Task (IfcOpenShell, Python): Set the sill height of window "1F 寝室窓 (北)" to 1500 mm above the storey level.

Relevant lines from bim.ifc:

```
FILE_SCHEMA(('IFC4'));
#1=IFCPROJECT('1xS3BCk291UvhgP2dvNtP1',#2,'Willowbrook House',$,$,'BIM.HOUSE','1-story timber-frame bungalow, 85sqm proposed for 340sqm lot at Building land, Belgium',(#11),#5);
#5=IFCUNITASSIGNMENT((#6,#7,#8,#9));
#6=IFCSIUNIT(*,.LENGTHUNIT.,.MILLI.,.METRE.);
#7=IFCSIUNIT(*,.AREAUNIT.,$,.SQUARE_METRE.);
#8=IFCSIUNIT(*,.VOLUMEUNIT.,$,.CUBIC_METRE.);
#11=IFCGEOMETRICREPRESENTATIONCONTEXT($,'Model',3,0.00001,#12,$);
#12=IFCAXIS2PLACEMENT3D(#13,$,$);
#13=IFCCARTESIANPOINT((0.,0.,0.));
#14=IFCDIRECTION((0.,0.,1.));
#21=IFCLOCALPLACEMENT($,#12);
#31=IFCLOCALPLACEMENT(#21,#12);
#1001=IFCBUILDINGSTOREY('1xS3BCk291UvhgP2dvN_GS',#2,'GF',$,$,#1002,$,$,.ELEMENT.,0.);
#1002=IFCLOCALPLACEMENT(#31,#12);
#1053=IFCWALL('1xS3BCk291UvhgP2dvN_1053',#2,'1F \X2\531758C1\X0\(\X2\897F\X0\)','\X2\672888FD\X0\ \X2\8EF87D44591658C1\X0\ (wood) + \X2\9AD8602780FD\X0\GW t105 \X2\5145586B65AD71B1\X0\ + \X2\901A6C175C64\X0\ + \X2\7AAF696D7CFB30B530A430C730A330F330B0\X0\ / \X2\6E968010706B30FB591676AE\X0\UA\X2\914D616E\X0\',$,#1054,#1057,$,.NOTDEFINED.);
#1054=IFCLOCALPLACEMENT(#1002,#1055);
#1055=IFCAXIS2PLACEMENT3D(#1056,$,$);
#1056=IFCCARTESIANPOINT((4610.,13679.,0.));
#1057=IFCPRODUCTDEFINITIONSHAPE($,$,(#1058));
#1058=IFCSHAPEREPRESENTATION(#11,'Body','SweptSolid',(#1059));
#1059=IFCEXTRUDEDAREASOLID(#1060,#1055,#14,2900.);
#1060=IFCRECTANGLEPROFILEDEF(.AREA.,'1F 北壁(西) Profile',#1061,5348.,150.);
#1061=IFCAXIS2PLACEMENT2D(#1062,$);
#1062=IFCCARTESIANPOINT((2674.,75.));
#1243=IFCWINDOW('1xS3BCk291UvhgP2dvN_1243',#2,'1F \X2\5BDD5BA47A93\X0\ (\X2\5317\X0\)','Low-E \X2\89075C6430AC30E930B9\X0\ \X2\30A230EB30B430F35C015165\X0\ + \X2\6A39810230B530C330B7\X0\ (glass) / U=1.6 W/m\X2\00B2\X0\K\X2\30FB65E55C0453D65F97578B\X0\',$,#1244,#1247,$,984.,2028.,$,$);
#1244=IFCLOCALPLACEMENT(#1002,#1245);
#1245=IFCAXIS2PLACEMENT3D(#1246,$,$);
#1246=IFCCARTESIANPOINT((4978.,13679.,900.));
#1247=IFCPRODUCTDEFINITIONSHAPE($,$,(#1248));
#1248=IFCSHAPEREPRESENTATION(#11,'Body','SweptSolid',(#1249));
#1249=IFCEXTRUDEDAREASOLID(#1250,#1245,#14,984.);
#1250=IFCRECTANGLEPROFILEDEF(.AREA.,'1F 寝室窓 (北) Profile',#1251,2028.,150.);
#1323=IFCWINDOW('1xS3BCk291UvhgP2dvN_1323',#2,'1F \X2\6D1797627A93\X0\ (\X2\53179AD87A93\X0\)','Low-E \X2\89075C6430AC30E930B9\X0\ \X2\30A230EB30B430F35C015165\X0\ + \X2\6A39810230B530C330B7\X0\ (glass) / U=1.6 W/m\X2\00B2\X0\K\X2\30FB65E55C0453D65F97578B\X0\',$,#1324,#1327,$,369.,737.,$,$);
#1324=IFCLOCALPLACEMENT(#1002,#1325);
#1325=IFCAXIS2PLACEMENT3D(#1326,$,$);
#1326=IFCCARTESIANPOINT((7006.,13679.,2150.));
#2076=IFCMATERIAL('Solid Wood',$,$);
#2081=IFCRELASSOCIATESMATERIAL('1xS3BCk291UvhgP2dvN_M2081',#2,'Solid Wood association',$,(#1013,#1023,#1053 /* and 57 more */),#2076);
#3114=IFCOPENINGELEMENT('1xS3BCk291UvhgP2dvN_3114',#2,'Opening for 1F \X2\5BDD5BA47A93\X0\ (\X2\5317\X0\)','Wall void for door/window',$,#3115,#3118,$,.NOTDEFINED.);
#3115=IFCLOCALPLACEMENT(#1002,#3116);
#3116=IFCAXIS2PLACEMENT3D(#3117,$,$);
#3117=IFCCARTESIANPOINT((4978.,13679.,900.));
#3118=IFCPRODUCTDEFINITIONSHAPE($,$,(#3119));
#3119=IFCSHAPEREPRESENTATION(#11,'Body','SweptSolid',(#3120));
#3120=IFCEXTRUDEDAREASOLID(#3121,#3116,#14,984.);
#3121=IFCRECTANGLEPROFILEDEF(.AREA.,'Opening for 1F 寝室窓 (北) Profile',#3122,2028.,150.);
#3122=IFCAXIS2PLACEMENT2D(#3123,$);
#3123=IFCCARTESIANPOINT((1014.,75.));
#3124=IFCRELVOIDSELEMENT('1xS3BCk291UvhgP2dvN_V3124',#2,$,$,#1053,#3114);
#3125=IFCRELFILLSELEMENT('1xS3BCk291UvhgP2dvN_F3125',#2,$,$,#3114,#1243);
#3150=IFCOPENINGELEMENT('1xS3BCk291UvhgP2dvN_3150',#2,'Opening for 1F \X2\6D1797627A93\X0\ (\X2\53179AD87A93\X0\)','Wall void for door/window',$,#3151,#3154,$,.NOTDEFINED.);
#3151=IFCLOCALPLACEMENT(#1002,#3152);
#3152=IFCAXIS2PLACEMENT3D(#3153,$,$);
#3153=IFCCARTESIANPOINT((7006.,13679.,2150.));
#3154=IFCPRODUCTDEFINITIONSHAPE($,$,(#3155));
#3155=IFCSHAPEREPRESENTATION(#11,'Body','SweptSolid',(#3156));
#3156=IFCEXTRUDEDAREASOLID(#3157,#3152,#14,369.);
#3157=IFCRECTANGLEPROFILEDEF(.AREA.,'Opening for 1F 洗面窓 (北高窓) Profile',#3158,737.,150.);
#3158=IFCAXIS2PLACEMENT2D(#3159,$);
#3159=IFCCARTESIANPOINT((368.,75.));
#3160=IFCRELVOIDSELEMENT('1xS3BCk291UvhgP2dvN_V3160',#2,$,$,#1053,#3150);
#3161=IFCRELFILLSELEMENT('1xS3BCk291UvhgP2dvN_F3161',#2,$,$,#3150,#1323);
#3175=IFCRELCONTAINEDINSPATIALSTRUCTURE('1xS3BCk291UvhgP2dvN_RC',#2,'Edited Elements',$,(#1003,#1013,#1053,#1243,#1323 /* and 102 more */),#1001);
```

```python
import numpy as np
import ifcopenshell
import ifcopenshell.api.geometry
import ifcopenshell.geom
import ifcopenshell.util.element
import ifcopenshell.util.placement
import ifcopenshell.util.shape
import ifcopenshell.util.unit

model = ifcopenshell.open("bim.ifc")
unit_scale = ifcopenshell.util.unit.calculate_unit_scale(model)

window = model.by_guid("1xS3BCk291UvhgP2dvN_1243")
opening = window.FillsVoids[0].RelatingOpeningElement
storey = ifcopenshell.util.element.get_container(window, ifc_class="IfcBuildingStorey")
level = ifcopenshell.util.placement.get_local_placement(storey.ObjectPlacement)[2, 3]

# The opening's origin need not be at the sill, so measure its lowest point.
shape = ifcopenshell.geom.create_shape(ifcopenshell.geom.settings(), opening)
bottom = ifcopenshell.util.shape.get_shape_bottom_elevation(shape, shape.geometry) / unit_scale
dz = level + 1.5 / unit_scale - bottom

shift = np.array([0.0, 0.0, dz])
# The window is not placed relative to its opening, so move both.
for product in (opening, window):
    matrix = ifcopenshell.util.placement.get_local_placement(product.ObjectPlacement)
    matrix[:3, 3] += shift
    ifcopenshell.api.geometry.edit_object_placement(model, product=product, matrix=matrix, is_si=False)

print(f"moved by {dz * unit_scale:+.3f} m")

model.write("bim_edited.ifc")
```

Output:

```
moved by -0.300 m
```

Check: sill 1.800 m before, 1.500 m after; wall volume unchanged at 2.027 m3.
